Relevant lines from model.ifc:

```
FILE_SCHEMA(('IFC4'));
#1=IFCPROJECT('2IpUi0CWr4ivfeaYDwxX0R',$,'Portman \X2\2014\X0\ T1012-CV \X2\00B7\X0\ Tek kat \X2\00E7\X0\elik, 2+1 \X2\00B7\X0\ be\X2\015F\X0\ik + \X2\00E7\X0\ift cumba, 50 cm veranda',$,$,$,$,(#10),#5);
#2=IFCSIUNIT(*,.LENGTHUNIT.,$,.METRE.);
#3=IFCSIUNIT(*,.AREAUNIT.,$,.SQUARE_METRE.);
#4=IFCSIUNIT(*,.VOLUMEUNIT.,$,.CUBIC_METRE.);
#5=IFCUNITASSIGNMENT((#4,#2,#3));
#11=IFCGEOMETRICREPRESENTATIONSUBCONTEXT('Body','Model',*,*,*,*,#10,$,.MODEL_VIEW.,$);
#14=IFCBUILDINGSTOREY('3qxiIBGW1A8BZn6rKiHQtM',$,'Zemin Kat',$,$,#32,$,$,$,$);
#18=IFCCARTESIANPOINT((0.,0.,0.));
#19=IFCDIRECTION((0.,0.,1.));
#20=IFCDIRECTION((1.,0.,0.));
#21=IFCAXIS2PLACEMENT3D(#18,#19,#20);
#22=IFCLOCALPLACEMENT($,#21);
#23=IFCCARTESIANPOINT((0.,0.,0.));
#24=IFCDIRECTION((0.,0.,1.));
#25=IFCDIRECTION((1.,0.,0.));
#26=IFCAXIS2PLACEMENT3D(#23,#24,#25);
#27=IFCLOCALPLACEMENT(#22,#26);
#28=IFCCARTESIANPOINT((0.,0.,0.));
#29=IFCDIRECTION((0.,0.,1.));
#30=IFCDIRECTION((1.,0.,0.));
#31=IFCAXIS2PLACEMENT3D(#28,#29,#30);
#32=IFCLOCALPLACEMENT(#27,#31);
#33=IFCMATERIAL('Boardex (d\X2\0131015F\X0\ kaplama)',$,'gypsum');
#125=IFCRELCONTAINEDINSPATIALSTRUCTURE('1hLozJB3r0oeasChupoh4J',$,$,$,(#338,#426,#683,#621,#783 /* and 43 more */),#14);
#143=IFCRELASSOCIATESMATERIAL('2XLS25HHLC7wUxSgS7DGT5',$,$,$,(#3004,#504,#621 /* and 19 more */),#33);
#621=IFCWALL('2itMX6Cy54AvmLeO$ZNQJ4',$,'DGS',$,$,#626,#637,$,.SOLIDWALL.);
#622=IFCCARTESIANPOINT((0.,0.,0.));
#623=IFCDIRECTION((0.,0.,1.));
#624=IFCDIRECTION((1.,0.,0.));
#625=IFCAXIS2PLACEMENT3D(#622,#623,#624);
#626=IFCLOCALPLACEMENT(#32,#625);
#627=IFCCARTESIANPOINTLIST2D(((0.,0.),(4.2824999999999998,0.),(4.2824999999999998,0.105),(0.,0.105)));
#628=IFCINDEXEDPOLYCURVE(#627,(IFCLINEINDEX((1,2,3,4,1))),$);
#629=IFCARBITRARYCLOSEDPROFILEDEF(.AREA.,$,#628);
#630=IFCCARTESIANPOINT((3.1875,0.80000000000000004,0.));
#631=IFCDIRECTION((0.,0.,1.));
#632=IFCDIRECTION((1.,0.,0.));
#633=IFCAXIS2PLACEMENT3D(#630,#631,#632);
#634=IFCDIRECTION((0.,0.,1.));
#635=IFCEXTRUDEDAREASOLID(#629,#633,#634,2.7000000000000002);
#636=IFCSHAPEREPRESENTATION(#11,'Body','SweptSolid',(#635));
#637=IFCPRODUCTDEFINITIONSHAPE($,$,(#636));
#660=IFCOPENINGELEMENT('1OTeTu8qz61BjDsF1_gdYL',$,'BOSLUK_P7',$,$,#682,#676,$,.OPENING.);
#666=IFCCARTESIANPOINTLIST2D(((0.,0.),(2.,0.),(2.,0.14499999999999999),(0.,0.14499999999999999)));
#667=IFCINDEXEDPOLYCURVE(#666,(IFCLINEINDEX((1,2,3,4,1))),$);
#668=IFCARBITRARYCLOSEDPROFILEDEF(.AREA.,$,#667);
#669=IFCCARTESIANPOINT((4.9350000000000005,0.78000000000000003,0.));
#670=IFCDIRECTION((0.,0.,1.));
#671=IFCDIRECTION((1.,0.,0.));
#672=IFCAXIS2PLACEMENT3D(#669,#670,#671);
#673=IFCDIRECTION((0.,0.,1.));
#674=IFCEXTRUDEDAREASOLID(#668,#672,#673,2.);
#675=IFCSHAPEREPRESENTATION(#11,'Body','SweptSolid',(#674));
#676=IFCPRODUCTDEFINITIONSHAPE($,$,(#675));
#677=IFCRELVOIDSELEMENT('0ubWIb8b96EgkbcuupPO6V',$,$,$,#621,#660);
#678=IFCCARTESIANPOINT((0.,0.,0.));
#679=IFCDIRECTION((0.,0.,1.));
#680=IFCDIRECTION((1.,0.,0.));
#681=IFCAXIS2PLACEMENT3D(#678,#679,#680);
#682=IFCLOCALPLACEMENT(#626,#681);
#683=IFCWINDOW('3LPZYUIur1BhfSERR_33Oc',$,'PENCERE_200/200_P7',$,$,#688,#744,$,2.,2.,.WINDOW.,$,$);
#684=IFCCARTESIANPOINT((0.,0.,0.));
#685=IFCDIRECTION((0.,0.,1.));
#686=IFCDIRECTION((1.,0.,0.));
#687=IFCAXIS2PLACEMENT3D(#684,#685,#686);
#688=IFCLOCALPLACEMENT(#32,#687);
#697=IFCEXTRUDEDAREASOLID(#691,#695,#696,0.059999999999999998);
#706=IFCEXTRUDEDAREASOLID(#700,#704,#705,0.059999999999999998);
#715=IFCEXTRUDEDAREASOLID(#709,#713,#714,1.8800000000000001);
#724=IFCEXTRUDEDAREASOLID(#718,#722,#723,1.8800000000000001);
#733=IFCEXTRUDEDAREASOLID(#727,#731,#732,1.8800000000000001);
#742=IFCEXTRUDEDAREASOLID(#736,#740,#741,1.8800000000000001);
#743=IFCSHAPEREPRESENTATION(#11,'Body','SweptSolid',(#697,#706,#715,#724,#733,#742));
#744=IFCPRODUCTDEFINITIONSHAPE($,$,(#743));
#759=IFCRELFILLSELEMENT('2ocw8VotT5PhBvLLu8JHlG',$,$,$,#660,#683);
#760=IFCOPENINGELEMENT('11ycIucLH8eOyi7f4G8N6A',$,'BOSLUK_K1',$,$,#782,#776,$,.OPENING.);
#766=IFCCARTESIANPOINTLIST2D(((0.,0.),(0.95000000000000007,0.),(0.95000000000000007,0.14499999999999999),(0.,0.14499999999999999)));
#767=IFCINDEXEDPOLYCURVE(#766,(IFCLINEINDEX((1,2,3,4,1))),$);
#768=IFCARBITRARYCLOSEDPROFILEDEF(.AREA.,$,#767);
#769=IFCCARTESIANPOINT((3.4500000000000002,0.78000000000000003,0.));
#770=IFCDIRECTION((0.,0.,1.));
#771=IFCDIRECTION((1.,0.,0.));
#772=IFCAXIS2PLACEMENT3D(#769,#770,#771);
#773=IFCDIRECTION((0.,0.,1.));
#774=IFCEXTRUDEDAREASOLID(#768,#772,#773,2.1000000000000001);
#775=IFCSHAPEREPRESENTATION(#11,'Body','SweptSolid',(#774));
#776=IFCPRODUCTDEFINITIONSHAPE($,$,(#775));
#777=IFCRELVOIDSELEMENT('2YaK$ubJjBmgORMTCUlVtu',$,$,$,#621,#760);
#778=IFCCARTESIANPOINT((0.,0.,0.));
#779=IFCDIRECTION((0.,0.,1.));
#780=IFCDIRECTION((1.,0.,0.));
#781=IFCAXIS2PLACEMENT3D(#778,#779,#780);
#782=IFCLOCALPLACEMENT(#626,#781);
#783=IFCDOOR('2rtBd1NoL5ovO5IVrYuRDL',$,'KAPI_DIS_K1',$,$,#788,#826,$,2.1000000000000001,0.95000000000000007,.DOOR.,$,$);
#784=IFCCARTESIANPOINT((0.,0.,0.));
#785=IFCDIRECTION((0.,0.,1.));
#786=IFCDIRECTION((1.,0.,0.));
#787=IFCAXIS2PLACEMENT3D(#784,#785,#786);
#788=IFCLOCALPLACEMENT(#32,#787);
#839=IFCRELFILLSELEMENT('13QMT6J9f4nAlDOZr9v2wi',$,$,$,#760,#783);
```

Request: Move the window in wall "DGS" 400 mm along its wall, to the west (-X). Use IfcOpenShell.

```python
import ifcopenshell
import ifcopenshell.api.geometry
import ifcopenshell.util.placement
import ifcopenshell.util.unit

model = ifcopenshell.open("model.ifc")
unit_scale = ifcopenshell.util.unit.calculate_unit_scale(model)

window = model.by_id(683)
opening = window.FillsVoids[0].RelatingOpeningElement
wall = opening.VoidsElements[0].RelatingBuildingElement

wall_matrix = ifcopenshell.util.placement.get_local_placement(wall.ObjectPlacement)
shift = wall_matrix[:3, 0] * -0.4 / unit_scale
before = ifcopenshell.util.placement.get_local_placement(window.ObjectPlacement)[:3, 3].copy()

# The window is not placed relative to its opening, so move both.
for product in (opening, window):
    matrix = ifcopenshell.util.placement.get_local_placement(product.ObjectPlacement)
    matrix[:3, 3] += shift
    ifcopenshell.api.geometry.edit_object_placement(model, product=product, matrix=matrix, is_si=False)

after = ifcopenshell.util.placement.get_local_placement(window.ObjectPlacement)[:3, 3]
print("window moved by", (after - before).round(3) + 0.0)

model.write("model_v2.ifc")
```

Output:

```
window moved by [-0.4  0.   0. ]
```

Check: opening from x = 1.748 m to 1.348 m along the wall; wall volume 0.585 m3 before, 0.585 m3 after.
